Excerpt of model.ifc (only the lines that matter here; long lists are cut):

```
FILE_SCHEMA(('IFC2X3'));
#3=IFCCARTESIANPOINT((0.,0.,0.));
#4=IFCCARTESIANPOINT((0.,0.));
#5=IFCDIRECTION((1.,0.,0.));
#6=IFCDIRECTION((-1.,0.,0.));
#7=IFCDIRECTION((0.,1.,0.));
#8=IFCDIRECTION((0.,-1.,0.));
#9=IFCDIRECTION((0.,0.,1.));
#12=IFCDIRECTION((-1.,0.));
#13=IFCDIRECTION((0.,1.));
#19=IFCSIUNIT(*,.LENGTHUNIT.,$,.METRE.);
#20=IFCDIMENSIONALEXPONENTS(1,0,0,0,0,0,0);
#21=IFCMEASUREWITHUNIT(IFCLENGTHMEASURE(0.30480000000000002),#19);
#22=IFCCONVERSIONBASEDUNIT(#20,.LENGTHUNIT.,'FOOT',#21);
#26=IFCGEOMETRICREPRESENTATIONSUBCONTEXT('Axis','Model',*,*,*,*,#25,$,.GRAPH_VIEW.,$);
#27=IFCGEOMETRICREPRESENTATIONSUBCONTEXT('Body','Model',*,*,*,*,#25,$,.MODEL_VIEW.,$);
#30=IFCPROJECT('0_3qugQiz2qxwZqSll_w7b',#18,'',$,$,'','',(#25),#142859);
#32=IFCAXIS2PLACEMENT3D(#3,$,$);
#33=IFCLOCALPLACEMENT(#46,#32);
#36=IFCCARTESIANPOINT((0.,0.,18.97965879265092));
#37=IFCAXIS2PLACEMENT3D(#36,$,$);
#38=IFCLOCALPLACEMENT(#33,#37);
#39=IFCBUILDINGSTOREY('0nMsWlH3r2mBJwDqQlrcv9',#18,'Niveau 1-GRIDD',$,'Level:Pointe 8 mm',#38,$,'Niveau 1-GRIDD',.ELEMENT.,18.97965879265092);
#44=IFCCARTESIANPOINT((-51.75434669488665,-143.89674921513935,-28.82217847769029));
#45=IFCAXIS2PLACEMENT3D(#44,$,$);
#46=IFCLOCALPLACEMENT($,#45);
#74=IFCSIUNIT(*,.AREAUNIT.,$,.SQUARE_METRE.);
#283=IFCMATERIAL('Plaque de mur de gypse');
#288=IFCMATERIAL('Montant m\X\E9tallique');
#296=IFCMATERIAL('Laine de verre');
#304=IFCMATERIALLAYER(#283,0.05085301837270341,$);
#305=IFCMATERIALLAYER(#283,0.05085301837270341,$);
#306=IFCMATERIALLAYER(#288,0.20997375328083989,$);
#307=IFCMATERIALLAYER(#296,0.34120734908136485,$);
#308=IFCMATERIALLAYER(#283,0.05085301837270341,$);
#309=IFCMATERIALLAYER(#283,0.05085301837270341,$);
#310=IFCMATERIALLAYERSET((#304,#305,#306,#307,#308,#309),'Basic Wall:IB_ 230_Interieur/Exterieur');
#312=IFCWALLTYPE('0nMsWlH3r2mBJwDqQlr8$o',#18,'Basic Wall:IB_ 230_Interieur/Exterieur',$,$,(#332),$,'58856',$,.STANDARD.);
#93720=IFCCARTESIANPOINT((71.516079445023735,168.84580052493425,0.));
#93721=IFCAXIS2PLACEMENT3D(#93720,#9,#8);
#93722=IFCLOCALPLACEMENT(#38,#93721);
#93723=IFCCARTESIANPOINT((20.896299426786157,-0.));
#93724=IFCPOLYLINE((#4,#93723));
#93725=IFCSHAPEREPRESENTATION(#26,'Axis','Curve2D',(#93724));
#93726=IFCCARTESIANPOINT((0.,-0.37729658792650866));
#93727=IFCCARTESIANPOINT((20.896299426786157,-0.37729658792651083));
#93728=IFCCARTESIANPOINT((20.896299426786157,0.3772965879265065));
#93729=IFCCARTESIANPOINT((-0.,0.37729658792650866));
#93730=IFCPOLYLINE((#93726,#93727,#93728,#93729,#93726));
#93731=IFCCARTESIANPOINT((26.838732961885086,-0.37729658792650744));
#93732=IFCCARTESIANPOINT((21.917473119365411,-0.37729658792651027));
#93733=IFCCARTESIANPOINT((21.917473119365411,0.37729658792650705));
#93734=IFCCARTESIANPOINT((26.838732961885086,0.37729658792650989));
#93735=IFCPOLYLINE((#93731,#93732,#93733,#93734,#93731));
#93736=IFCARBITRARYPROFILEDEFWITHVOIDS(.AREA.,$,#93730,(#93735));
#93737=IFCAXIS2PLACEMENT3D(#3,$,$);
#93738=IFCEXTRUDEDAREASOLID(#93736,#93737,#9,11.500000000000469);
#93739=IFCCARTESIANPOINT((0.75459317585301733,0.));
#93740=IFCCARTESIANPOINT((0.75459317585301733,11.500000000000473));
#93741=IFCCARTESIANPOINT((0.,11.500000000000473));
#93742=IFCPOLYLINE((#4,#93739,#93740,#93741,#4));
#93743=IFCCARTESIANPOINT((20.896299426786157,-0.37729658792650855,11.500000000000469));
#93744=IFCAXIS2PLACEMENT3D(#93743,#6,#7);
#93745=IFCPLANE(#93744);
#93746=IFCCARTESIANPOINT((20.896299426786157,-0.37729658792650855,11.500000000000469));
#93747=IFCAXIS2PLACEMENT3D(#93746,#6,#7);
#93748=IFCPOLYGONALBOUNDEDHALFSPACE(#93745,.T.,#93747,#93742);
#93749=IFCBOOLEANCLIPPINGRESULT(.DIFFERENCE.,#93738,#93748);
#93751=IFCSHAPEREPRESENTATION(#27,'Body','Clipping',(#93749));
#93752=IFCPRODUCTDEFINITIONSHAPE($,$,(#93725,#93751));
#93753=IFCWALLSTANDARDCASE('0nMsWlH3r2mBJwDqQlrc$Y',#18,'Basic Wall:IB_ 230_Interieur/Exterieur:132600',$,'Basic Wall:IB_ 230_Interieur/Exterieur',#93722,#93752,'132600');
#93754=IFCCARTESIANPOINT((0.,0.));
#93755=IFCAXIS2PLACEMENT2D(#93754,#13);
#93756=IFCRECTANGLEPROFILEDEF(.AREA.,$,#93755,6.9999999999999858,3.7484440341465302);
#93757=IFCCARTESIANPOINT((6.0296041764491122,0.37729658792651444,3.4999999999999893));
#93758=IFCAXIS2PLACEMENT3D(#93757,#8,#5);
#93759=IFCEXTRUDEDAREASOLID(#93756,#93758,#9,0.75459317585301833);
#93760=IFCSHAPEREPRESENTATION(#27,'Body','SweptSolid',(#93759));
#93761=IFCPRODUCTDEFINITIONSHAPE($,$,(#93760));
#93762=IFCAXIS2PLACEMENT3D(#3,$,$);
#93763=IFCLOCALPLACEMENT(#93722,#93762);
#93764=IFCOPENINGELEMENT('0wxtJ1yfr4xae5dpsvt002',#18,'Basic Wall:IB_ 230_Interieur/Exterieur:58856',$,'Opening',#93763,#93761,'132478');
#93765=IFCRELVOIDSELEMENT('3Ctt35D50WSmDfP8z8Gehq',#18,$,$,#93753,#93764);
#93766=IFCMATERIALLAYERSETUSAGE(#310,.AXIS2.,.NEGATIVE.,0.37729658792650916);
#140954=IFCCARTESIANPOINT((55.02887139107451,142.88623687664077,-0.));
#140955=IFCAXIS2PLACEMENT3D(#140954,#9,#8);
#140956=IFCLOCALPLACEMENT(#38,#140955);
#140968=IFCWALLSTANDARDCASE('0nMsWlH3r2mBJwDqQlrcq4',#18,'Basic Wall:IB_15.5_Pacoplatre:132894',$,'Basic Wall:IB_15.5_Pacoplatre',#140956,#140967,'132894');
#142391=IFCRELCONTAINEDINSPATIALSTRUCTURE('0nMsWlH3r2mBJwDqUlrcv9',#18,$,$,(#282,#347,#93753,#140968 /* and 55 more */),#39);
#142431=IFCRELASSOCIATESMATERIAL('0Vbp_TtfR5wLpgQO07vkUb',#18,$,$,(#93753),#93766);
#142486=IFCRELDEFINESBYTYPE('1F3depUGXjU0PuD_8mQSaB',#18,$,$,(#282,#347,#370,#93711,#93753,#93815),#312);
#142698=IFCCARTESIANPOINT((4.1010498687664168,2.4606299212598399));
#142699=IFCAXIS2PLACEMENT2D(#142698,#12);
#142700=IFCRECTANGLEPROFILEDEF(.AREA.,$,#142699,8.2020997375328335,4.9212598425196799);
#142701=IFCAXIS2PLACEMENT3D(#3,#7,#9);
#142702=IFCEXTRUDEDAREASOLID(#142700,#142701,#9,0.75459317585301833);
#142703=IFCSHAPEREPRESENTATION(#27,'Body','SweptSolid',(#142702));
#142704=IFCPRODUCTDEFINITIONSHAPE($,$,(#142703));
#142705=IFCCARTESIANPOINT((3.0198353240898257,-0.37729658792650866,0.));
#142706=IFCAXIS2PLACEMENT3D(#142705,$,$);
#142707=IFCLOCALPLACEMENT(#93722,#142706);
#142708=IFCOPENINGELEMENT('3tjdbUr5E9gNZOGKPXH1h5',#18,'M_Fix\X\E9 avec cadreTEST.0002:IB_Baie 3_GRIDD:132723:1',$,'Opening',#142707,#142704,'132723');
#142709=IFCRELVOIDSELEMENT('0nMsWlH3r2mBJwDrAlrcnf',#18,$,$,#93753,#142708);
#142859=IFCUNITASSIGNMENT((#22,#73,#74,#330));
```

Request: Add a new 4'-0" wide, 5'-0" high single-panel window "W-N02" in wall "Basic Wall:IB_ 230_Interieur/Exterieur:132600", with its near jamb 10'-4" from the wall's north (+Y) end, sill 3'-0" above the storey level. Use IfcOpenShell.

```python
import numpy as np
import ifcopenshell
import ifcopenshell.api.feature
import ifcopenshell.api.geometry
import ifcopenshell.api.root
import ifcopenshell.api.spatial
import ifcopenshell.api.type
import ifcopenshell.geom
import ifcopenshell.util.element
import ifcopenshell.util.placement
import ifcopenshell.util.representation
import ifcopenshell.util.shape
import ifcopenshell.util.unit

model = ifcopenshell.open("model.ifc")
unit_scale = ifcopenshell.util.unit.calculate_unit_scale(model)
settings = ifcopenshell.geom.settings()


def volume(element):
    """Net volume in cubic metres, openings subtracted."""
    shape = ifcopenshell.geom.create_shape(settings, element)
    return ifcopenshell.util.shape.get_volume(shape.geometry)


wall = model.by_guid("0nMsWlH3r2mBJwDqQlrc$Y")
storey = ifcopenshell.util.element.get_container(wall, ifc_class="IfcBuildingStorey")
context = ifcopenshell.util.representation.get_context(model, "Model", "Body", "MODEL_VIEW")
before = volume(wall)

width, height, from_end, sill = 1.2192, 1.524, 3.1496, 0.9144  # metres

# The wall runs along its own X axis, and the end named is its -X end.
wall_shape = ifcopenshell.geom.create_shape(settings, wall)
x, y, z = ifcopenshell.util.shape.get_vertices(wall_shape.geometry).T
start = x.min() + from_end
face, thickness = float(y.min()), float(y.max() - y.min())
wall_matrix = ifcopenshell.util.placement.get_local_placement(wall.ObjectPlacement)
level = ifcopenshell.util.placement.get_local_placement(storey.ObjectPlacement)[2, 3]


def in_wall(x, y):
    """Placement at x, y metres in the wall's axes, at sill height."""
    matrix = wall_matrix.copy()
    matrix[:, 3] = wall_matrix @ np.array([x / unit_scale, y / unit_scale, 0.0, 1.0])
    matrix[2, 3] = level + sill / unit_scale
    return matrix


# Opening: a box that overshoots both wall faces by 50 mm.
opening = ifcopenshell.api.root.create_entity(model, ifc_class="IfcOpeningElement")
box = ifcopenshell.api.geometry.add_wall_representation(
    model, context=context, length=width, height=height, thickness=thickness + 0.1
)
ifcopenshell.api.geometry.assign_representation(model, product=opening, representation=box)
ifcopenshell.api.geometry.edit_object_placement(model, product=opening, matrix=in_wall(start, face - 0.05), is_si=False)
ifcopenshell.api.feature.add_feature(model, feature=opening, element=wall)

window = ifcopenshell.api.root.create_entity(model, ifc_class="IfcWindow", name="W-N02")
window.OverallWidth, window.OverallHeight = width / unit_scale, height / unit_scale
body = ifcopenshell.api.geometry.add_window_representation(
    model,
    context=context,
    overall_width=window.OverallWidth,
    overall_height=window.OverallHeight,
    partition_type="SINGLE_PANEL",
)
ifcopenshell.api.geometry.assign_representation(model, product=window, representation=body)
ifcopenshell.api.spatial.assign_container(model, products=[window], relating_structure=storey)
fills = ifcopenshell.api.feature.add_filling(model, opening=opening, element=window)
fills.OwnerHistory = window.OwnerHistory  # required in IFC2X3

# IFC2X3 keeps the operation on the window style.
style = ifcopenshell.api.root.create_entity(model, ifc_class="IfcWindowStyle", name="W-N02")
style.OperationType, style.ConstructionType = "SINGLE_PANEL", "NOTDEFINED"
style.ParameterTakesPrecedence = style.Sizeable = False
ifcopenshell.api.type.assign_type(model, related_objects=[window], relating_type=style)

# Centre the window in the wall's thickness.
ifcopenshell.api.geometry.edit_object_placement(model, product=window, matrix=in_wall(start, face), is_si=False)
window_shape = ifcopenshell.geom.create_shape(settings, window)
depth = ifcopenshell.util.shape.get_vertices(window_shape.geometry)[:, 1]
offset = face + thickness / 2 - (depth.min() + depth.max()) / 2
ifcopenshell.api.geometry.edit_object_placement(model, product=window, matrix=in_wall(start, offset), is_si=False)

after = volume(wall)

print(f"wall volume {before:.3f} -> {after:.3f} m3")

model.write("model_rev.ifc")
```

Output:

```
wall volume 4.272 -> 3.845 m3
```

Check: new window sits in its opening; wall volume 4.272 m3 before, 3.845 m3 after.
